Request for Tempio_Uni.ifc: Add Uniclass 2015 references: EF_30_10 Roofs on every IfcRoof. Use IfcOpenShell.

First a look at what the model holds.

```python
import ifcopenshell

model = ifcopenshell.open("Tempio_Uni.ifc")
print(model.schema)
print("classifications:", [c.Name for c in model.by_type("IfcClassification")])
for ifc_class in ("IfcDoor", "IfcRoof", "IfcStair", "IfcWall", "IfcWindow"):
    print(ifc_class, len(model.by_type(ifc_class)))
```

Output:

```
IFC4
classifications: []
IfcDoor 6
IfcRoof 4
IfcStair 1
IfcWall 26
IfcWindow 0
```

```python
import ifcopenshell
import ifcopenshell.api.classification

model = ifcopenshell.open("Tempio_Uni.ifc")

system = ifcopenshell.api.classification.add_classification(model, classification="Uniclass 2015")

codes = {
    "IfcRoof": ("EF_30_10", "Roofs"),
}
for ifc_class, (code, name) in codes.items():
    products = model.by_type(ifc_class)
    ifcopenshell.api.classification.add_reference(
        model, products=products, classification=system, identification=code, name=name
    )
    print(code, len(products))

model.write("Tempio_Uni_edited.ifc")
```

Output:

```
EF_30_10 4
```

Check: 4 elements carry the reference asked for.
